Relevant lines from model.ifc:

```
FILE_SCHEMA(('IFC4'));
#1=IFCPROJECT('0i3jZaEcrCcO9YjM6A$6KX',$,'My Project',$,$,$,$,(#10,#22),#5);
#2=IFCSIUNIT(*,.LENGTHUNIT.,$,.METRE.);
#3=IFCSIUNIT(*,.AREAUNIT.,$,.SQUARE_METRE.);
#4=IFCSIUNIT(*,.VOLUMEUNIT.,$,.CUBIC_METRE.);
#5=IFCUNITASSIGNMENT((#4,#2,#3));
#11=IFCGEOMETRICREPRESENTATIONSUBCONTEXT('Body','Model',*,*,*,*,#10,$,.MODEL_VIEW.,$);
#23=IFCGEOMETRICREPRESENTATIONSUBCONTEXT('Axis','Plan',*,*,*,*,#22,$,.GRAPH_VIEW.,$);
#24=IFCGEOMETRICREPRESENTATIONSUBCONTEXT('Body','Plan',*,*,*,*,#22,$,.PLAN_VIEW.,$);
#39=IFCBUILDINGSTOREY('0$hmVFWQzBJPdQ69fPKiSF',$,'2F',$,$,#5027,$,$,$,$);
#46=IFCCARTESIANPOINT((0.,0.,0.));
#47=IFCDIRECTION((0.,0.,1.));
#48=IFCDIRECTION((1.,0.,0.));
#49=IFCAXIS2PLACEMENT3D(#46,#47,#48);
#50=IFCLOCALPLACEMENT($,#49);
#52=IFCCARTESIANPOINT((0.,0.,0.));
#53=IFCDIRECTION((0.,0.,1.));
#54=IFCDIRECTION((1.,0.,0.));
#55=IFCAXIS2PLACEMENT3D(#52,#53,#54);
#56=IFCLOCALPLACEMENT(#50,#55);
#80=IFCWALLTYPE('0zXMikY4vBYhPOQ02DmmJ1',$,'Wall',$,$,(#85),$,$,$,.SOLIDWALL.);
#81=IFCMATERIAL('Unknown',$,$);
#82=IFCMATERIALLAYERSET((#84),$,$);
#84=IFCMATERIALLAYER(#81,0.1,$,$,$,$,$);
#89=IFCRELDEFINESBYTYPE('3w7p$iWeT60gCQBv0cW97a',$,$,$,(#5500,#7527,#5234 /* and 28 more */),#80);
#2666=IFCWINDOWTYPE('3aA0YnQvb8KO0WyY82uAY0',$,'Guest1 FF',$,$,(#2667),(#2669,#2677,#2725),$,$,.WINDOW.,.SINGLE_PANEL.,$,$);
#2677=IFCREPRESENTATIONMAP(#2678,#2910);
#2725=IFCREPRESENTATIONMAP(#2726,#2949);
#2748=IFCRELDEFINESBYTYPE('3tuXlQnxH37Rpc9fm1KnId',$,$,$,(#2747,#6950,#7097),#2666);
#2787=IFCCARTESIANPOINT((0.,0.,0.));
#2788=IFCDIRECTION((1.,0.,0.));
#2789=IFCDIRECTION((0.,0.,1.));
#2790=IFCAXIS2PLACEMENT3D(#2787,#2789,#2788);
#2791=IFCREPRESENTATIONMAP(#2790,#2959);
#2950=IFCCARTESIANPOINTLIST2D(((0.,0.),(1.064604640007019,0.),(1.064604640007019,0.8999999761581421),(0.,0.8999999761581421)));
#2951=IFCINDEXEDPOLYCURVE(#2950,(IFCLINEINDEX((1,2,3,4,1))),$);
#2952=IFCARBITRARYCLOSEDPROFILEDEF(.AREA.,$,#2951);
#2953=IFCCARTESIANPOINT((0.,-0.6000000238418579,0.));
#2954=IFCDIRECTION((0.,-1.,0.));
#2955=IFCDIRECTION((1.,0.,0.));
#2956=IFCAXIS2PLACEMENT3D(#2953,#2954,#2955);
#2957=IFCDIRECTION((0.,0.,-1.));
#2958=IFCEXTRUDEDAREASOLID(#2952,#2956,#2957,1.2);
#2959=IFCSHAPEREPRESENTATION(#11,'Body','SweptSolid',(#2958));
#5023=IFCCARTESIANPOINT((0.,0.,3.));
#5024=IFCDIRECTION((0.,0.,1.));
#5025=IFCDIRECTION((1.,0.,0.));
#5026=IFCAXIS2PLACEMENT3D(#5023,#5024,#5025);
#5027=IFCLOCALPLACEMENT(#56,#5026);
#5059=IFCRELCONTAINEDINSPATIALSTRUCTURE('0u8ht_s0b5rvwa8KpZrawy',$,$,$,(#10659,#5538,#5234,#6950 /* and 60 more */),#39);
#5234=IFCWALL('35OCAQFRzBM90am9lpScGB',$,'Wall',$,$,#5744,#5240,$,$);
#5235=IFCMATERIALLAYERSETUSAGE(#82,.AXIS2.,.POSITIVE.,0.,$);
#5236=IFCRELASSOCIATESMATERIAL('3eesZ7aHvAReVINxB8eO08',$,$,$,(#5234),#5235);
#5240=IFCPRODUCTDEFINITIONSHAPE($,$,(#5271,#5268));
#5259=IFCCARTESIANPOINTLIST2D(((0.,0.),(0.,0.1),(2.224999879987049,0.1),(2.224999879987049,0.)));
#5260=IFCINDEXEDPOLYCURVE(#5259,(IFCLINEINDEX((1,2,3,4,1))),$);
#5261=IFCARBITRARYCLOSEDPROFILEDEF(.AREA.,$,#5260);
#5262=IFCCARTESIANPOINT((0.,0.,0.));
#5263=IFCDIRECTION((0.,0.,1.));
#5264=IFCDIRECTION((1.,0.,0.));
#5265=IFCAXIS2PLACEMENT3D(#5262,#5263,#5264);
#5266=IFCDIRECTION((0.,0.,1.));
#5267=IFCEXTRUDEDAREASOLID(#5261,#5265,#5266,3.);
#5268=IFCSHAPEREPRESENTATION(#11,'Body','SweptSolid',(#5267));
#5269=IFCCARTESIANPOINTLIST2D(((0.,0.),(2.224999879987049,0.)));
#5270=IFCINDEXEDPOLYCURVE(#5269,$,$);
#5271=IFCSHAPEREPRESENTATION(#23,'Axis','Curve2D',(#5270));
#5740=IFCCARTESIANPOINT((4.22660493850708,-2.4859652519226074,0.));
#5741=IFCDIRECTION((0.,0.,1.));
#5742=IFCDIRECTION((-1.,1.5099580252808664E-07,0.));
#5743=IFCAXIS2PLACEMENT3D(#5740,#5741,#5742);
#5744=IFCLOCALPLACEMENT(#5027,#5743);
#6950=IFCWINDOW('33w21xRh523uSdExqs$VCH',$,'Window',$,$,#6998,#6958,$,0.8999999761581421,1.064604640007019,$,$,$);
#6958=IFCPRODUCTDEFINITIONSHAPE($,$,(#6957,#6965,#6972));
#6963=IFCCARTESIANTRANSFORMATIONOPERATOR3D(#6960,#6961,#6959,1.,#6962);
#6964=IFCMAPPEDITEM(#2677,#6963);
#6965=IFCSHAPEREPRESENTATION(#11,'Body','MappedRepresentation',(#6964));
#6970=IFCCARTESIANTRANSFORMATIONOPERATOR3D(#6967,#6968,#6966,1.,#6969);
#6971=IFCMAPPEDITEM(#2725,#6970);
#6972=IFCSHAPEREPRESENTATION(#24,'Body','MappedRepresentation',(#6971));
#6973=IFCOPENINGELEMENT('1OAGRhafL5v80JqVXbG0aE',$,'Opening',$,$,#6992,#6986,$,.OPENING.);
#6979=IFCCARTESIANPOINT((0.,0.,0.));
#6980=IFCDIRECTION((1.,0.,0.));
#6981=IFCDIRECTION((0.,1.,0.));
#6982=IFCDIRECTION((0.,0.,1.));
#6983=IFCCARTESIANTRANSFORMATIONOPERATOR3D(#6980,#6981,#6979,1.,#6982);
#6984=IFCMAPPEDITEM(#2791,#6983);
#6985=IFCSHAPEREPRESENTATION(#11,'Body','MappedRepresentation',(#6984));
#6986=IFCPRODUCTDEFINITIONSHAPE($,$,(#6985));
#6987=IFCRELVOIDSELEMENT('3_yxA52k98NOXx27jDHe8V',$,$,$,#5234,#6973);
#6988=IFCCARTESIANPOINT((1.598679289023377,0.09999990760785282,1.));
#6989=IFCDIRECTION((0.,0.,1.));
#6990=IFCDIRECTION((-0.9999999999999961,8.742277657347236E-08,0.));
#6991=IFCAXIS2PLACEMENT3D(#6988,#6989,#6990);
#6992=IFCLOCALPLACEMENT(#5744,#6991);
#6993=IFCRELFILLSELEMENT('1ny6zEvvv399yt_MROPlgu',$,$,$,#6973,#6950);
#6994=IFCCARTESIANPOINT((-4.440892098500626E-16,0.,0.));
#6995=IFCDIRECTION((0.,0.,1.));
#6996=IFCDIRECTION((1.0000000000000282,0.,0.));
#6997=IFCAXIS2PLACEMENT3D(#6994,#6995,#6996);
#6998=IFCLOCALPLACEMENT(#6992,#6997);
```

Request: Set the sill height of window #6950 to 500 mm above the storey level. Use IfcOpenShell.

```python
import numpy as np
import ifcopenshell
import ifcopenshell.api.geometry
import ifcopenshell.geom
import ifcopenshell.util.element
import ifcopenshell.util.placement
import ifcopenshell.util.shape
import ifcopenshell.util.unit

model = ifcopenshell.open("model.ifc")
unit_scale = ifcopenshell.util.unit.calculate_unit_scale(model)

window = model.by_guid("33w21xRh523uSdExqs$VCH")
opening = window.FillsVoids[0].RelatingOpeningElement
storey = ifcopenshell.util.element.get_container(window, ifc_class="IfcBuildingStorey")
level = ifcopenshell.util.placement.get_local_placement(storey.ObjectPlacement)[2, 3]

# The opening's origin need not be at the sill, so measure its lowest point.
shape = ifcopenshell.geom.create_shape(ifcopenshell.geom.settings(), opening)
bottom = ifcopenshell.util.shape.get_shape_bottom_elevation(shape, shape.geometry) / unit_scale
dz = level + 0.5 / unit_scale - bottom

shift = np.array([0.0, 0.0, dz])
# The window is placed relative to its opening, so it follows when the opening moves.
matrix = ifcopenshell.util.placement.get_local_placement(opening.ObjectPlacement)
matrix[:3, 3] += shift
ifcopenshell.api.geometry.edit_object_placement(
    model, product=opening, matrix=matrix, is_si=False, should_transform_children=True
)

print(f"moved by {dz * unit_scale:+.3f} m")

model.write("model_rev.ifc")
```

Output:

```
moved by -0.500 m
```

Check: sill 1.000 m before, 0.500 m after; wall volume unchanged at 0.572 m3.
